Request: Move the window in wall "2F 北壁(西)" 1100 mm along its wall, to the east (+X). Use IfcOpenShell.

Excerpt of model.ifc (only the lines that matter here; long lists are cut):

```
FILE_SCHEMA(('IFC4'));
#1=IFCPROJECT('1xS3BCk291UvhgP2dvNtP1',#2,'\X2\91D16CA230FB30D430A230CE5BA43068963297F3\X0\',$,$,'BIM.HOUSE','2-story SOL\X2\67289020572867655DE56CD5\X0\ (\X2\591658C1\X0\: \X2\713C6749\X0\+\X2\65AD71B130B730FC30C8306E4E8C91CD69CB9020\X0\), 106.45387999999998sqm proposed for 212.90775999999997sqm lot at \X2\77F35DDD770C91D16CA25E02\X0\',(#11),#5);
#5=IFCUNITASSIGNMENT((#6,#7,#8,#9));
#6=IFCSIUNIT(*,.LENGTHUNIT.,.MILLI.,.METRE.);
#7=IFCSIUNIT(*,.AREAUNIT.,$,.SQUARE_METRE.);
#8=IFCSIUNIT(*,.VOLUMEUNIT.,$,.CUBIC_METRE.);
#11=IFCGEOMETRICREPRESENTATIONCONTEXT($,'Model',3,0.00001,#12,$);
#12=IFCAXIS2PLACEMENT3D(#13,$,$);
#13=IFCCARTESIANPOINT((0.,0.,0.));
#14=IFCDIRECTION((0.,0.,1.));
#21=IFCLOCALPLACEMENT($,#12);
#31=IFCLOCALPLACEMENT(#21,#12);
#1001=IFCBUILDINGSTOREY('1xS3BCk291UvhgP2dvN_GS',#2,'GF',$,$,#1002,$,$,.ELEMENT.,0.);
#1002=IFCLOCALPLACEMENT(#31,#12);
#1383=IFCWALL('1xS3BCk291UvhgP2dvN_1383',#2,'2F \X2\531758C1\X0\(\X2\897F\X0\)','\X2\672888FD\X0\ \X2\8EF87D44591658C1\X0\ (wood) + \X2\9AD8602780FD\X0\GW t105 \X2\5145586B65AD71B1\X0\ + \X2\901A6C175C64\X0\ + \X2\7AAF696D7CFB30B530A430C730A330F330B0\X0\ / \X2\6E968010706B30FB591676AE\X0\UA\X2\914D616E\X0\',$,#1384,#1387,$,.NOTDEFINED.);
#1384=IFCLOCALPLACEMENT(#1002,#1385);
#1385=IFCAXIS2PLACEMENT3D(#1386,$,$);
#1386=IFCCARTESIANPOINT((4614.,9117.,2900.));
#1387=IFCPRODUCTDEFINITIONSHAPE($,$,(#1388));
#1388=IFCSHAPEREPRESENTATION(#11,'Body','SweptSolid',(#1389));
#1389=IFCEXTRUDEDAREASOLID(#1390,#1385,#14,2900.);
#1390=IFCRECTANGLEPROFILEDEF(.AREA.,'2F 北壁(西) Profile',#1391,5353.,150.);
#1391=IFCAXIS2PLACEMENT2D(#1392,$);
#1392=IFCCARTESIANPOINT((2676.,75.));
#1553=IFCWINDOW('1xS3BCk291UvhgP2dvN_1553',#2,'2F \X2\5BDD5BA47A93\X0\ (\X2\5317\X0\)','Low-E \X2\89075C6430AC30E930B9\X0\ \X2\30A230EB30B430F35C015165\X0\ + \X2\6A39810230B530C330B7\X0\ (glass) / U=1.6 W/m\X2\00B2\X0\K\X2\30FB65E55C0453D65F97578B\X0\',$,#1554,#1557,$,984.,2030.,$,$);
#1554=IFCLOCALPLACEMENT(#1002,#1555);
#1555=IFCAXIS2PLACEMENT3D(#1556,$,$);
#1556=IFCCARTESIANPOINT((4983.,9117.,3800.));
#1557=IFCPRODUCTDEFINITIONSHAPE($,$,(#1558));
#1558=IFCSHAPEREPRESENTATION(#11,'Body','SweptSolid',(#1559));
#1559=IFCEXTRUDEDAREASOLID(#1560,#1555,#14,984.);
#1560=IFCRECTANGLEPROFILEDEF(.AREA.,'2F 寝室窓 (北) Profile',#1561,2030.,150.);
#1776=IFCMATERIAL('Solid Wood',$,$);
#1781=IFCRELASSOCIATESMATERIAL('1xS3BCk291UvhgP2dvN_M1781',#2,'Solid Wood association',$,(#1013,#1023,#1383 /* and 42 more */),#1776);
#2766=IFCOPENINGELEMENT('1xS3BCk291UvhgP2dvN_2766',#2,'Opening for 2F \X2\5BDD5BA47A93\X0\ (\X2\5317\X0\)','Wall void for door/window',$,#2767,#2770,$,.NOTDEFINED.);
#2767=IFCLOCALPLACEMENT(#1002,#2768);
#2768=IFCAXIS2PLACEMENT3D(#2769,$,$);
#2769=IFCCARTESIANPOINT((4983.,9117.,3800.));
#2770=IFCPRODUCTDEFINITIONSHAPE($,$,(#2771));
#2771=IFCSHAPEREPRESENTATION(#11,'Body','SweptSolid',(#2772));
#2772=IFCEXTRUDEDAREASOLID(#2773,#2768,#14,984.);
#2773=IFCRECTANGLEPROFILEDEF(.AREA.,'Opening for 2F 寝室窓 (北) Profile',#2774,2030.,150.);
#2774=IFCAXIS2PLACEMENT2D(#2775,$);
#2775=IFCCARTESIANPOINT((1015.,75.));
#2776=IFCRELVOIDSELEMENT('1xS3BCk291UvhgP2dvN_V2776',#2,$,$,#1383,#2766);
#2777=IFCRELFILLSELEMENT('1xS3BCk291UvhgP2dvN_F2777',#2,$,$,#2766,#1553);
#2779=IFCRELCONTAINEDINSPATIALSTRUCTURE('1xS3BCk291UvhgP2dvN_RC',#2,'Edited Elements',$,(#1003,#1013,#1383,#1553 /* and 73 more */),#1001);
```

```python
import ifcopenshell
import ifcopenshell.api.geometry
import ifcopenshell.util.placement
import ifcopenshell.util.unit

model = ifcopenshell.open("model.ifc")
unit_scale = ifcopenshell.util.unit.calculate_unit_scale(model)

window = model.by_id(1553)
opening = window.FillsVoids[0].RelatingOpeningElement
wall = opening.VoidsElements[0].RelatingBuildingElement

wall_matrix = ifcopenshell.util.placement.get_local_placement(wall.ObjectPlacement)
shift = wall_matrix[:3, 0] * 1.1 / unit_scale
before = ifcopenshell.util.placement.get_local_placement(window.ObjectPlacement)[:3, 3].copy()

# The window is not placed relative to its opening, so move both.
for product in (opening, window):
    matrix = ifcopenshell.util.placement.get_local_placement(product.ObjectPlacement)
    matrix[:3, 3] += shift
    ifcopenshell.api.geometry.edit_object_placement(model, product=product, matrix=matrix, is_si=False)

after = ifcopenshell.util.placement.get_local_placement(window.ObjectPlacement)[:3, 3]
print("window moved by", (after - before).round(3) + 0.0)

model.write("model_edited.ifc")
```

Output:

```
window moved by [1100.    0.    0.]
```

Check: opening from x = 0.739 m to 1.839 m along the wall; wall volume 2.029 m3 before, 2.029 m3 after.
